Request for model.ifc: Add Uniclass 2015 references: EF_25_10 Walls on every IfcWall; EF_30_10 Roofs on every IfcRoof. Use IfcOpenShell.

First a look at what the model holds.

```python
import ifcopenshell

model = ifcopenshell.open("model.ifc")
print(model.schema)
print("classifications:", [c.Name for c in model.by_type("IfcClassification")])
for ifc_class in ("IfcDoor", "IfcRoof", "IfcStair", "IfcWall", "IfcWindow"):
    print(ifc_class, len(model.by_type(ifc_class)))
```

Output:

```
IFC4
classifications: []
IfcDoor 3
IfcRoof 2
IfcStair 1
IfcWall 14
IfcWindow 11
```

```python
import ifcopenshell
import ifcopenshell.api.classification

model = ifcopenshell.open("model.ifc")

system = ifcopenshell.api.classification.add_classification(model, classification="Uniclass 2015")

codes = {
    "IfcWall": ("EF_25_10", "Walls"),
    "IfcRoof": ("EF_30_10", "Roofs"),
}
for ifc_class, (code, name) in codes.items():
    products = model.by_type(ifc_class)
    ifcopenshell.api.classification.add_reference(
        model, products=products, classification=system, identification=code, name=name
    )
    print(code, len(products))

model.write("model_edited.ifc")
```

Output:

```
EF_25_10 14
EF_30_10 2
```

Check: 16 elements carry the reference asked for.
